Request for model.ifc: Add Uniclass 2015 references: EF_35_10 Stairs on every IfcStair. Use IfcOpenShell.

First a look at what the model holds.

```python
import ifcopenshell

model = ifcopenshell.open("model.ifc")
print(model.schema)
print("classifications:", [c.Name for c in model.by_type("IfcClassification")])
for ifc_class in ("IfcDoor", "IfcRoof", "IfcStair", "IfcWall", "IfcWindow"):
    print(ifc_class, len(model.by_type(ifc_class)))
```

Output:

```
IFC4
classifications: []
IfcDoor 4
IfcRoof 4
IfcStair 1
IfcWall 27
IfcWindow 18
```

```python
import ifcopenshell
import ifcopenshell.api.classification

model = ifcopenshell.open("model.ifc")

system = ifcopenshell.api.classification.add_classification(model, classification="Uniclass 2015")

codes = {
    "IfcStair": ("EF_35_10", "Stairs"),
}
for ifc_class, (code, name) in codes.items():
    products = model.by_type(ifc_class)
    ifcopenshell.api.classification.add_reference(
        model, products=products, classification=system, identification=code, name=name
    )
    print(code, len(products))

model.write("model_updated.ifc")
```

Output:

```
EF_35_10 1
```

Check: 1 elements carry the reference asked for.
